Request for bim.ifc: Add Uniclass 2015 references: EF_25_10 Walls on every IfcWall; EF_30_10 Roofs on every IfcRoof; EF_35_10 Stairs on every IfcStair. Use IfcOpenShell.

First a look at what the model holds.

```python
import ifcopenshell

model = ifcopenshell.open("bim.ifc")
print(model.schema)
print("classifications:", [c.Name for c in model.by_type("IfcClassification")])
for ifc_class in ("IfcDoor", "IfcRoof", "IfcStair", "IfcWall", "IfcWindow"):
    print(ifc_class, len(model.by_type(ifc_class)))
```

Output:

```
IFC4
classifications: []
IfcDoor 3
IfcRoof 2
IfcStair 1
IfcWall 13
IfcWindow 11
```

```python
import ifcopenshell
import ifcopenshell.api.classification

model = ifcopenshell.open("bim.ifc")

system = ifcopenshell.api.classification.add_classification(model, classification="Uniclass 2015")

codes = {
    "IfcWall": ("EF_25_10", "Walls"),
    "IfcRoof": ("EF_30_10", "Roofs"),
    "IfcStair": ("EF_35_10", "Stairs"),
}
for ifc_class, (code, name) in codes.items():
    products = model.by_type(ifc_class)
    ifcopenshell.api.classification.add_reference(
        model, products=products, classification=system, identification=code, name=name
    )
    print(code, len(products))

model.write("bim_edited.ifc")
```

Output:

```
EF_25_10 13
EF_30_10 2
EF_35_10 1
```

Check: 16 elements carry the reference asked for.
